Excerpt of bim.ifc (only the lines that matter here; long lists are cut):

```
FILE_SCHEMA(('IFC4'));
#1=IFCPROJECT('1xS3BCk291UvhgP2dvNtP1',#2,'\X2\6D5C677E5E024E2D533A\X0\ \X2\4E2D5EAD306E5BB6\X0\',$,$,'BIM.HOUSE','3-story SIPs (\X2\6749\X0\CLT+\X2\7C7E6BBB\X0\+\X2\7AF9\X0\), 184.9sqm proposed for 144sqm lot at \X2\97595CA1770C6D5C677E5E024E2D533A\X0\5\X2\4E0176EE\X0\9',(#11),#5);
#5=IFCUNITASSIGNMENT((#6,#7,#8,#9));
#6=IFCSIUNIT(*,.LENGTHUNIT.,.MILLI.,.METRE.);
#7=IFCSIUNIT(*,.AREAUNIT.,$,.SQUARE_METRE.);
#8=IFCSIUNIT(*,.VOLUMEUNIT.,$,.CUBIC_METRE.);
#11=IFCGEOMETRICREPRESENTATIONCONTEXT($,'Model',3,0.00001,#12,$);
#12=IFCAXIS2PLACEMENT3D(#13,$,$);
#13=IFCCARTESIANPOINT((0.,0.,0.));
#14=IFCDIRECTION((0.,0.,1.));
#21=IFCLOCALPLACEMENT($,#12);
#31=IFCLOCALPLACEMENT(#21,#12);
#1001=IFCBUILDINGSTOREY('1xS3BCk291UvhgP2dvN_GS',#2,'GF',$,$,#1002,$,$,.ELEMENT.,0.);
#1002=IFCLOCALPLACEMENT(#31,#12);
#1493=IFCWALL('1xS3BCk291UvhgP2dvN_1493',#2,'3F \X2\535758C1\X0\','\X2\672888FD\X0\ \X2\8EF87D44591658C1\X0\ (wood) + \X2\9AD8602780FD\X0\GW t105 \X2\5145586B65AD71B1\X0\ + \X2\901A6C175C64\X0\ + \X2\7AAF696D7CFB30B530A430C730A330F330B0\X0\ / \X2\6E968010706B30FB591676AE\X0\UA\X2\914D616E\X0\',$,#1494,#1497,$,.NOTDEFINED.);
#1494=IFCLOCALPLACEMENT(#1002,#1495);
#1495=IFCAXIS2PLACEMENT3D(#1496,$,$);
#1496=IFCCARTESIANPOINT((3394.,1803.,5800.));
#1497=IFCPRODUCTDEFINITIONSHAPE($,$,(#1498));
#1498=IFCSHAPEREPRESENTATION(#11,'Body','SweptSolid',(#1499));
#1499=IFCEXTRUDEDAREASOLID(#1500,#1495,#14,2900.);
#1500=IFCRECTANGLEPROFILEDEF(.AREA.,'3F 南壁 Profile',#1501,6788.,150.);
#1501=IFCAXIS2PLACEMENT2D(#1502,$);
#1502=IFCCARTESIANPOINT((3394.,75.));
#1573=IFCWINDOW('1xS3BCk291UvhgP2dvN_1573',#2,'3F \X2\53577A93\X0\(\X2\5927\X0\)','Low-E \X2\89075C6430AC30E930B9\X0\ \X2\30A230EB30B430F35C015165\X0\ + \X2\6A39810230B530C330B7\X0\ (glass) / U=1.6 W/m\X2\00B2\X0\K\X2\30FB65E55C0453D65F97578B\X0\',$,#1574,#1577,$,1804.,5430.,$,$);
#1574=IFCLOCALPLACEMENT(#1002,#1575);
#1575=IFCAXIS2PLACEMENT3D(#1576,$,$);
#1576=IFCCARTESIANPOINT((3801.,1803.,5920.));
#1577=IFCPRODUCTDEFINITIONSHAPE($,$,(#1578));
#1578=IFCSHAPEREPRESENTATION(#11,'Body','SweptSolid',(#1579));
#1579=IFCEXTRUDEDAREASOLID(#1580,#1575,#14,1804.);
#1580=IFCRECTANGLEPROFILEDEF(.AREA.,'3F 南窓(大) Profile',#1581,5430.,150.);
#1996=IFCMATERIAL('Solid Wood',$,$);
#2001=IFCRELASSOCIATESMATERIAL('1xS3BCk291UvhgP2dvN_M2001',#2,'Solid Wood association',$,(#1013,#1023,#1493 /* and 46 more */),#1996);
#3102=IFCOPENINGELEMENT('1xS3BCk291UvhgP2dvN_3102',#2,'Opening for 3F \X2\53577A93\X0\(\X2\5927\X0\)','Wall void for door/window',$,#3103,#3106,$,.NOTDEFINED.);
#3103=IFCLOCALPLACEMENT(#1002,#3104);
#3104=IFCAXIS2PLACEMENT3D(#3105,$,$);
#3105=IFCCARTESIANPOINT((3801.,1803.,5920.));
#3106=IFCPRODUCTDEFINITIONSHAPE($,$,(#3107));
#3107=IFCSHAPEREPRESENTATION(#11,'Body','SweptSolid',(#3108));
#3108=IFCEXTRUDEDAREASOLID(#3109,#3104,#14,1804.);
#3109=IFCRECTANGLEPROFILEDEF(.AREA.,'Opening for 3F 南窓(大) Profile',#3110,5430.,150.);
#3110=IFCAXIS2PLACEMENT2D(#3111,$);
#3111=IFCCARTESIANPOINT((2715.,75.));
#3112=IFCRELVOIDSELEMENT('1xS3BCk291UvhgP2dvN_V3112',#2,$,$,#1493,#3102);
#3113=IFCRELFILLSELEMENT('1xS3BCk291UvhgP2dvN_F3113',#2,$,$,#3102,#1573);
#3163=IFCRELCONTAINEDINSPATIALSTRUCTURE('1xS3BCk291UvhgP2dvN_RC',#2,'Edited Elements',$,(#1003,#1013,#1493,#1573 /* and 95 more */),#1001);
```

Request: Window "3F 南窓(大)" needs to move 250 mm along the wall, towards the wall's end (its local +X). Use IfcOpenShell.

```python
import ifcopenshell
import ifcopenshell.api.geometry
import ifcopenshell.util.placement

model = ifcopenshell.open("bim.ifc")

window = model.by_guid("1xS3BCk291UvhgP2dvN_1573")
opening = window.FillsVoids[0].RelatingOpeningElement
wall = opening.VoidsElements[0].RelatingBuildingElement

wall_matrix = ifcopenshell.util.placement.get_local_placement(wall.ObjectPlacement)
shift = wall_matrix[:3, 0] * 250.0
before = ifcopenshell.util.placement.get_local_placement(window.ObjectPlacement)[:3, 3].copy()

# The window is not placed relative to its opening, so move both.
for product in (opening, window):
    matrix = ifcopenshell.util.placement.get_local_placement(product.ObjectPlacement)
    matrix[:3, 3] += shift
    ifcopenshell.api.geometry.edit_object_placement(model, product=product, matrix=matrix, is_si=False)

after = ifcopenshell.util.placement.get_local_placement(window.ObjectPlacement)[:3, 3]
print("window moved by", (after - before).round(3) + 0.0)

model.write("bim_edited.ifc")
```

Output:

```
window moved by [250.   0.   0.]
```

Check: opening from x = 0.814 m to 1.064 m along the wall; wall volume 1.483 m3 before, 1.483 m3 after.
